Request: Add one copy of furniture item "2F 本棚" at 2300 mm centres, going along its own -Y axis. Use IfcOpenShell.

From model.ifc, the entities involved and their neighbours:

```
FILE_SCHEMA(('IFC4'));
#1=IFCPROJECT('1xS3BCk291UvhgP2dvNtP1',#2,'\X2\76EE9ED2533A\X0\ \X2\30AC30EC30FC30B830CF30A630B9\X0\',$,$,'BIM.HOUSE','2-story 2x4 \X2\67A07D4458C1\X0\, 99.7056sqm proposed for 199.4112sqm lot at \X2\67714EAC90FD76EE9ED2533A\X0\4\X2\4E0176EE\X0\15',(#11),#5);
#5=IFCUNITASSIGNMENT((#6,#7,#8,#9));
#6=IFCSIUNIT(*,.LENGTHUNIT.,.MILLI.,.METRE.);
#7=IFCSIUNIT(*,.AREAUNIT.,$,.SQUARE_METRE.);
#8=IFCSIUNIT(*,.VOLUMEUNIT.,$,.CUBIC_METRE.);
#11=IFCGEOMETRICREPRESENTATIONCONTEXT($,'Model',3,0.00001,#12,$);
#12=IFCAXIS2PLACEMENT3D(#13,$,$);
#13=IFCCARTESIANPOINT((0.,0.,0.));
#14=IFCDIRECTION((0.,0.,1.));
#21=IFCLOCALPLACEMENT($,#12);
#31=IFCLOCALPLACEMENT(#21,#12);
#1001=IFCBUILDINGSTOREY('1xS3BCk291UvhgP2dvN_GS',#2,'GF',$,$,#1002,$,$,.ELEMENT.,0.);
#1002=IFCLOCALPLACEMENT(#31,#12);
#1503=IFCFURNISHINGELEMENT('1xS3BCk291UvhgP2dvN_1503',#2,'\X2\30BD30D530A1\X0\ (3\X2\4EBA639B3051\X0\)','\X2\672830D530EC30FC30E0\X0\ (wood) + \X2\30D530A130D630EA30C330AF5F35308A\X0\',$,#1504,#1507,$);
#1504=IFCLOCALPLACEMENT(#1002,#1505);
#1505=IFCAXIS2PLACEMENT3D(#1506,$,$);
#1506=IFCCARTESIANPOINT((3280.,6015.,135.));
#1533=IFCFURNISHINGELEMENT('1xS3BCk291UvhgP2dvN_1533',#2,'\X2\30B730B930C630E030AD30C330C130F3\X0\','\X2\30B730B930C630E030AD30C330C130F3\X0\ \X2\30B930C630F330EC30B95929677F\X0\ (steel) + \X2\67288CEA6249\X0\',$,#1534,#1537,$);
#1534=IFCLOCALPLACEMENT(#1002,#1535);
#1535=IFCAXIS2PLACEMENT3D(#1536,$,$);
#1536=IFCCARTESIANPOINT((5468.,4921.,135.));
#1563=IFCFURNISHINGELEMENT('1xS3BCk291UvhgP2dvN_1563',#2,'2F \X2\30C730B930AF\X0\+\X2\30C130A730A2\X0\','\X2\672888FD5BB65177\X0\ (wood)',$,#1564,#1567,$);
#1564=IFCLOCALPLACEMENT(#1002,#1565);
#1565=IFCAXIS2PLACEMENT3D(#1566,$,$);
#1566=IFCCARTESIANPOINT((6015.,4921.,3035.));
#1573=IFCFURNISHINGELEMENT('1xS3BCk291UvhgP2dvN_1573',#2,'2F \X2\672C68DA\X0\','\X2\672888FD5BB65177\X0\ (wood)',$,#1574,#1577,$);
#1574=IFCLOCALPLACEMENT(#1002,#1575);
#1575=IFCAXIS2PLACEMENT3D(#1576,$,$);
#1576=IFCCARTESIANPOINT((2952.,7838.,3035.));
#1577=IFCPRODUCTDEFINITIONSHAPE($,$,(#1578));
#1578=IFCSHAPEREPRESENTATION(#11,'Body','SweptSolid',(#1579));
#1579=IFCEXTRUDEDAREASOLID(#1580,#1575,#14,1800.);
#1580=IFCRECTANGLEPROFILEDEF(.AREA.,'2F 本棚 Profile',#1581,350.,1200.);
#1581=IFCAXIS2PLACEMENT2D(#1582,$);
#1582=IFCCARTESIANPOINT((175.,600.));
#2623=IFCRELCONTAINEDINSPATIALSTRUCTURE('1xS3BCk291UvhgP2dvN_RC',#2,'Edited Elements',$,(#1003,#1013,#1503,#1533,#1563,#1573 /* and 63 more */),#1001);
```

```python
import ifcopenshell
import ifcopenshell.api.geometry
import ifcopenshell.api.root
import ifcopenshell.util.element
import ifcopenshell.util.placement
import ifcopenshell.util.unit

model = ifcopenshell.open("model.ifc")
unit_scale = ifcopenshell.util.unit.calculate_unit_scale(model)


def reuse_history(source, copy):
    """copy_class also copies each property set's owner history, people and application; keep the originals."""
    for rel in copy.IsDefinedBy:
        if rel.is_a("IfcRelDefinesByProperties") and (history := rel.RelatingPropertyDefinition.OwnerHistory):
            rel.RelatingPropertyDefinition.OwnerHistory = source.OwnerHistory
            ifcopenshell.util.element.remove_deep2(model, history)


source = model.by_id(1573)
base = ifcopenshell.util.placement.get_local_placement(source.ObjectPlacement)
step = -base[:3, 1] * 2.3 / unit_scale

for i in range(1, 2):
    copy = ifcopenshell.api.root.copy_class(model, product=source)
    copy.Representation = ifcopenshell.util.element.copy_deep(
        model, source.Representation, exclude=["IfcGeometricRepresentationContext", "IfcRepresentationMap"]
    )
    reuse_history(source, copy)
    matrix = base.copy()
    matrix[:3, 3] += i * step
    print("added at", matrix[:3, 3].round(3) + 0.0)
    ifcopenshell.api.geometry.edit_object_placement(model, product=copy, matrix=matrix, is_si=False)

model.write("model_updated.ifc")
```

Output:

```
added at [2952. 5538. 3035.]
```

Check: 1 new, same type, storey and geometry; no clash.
